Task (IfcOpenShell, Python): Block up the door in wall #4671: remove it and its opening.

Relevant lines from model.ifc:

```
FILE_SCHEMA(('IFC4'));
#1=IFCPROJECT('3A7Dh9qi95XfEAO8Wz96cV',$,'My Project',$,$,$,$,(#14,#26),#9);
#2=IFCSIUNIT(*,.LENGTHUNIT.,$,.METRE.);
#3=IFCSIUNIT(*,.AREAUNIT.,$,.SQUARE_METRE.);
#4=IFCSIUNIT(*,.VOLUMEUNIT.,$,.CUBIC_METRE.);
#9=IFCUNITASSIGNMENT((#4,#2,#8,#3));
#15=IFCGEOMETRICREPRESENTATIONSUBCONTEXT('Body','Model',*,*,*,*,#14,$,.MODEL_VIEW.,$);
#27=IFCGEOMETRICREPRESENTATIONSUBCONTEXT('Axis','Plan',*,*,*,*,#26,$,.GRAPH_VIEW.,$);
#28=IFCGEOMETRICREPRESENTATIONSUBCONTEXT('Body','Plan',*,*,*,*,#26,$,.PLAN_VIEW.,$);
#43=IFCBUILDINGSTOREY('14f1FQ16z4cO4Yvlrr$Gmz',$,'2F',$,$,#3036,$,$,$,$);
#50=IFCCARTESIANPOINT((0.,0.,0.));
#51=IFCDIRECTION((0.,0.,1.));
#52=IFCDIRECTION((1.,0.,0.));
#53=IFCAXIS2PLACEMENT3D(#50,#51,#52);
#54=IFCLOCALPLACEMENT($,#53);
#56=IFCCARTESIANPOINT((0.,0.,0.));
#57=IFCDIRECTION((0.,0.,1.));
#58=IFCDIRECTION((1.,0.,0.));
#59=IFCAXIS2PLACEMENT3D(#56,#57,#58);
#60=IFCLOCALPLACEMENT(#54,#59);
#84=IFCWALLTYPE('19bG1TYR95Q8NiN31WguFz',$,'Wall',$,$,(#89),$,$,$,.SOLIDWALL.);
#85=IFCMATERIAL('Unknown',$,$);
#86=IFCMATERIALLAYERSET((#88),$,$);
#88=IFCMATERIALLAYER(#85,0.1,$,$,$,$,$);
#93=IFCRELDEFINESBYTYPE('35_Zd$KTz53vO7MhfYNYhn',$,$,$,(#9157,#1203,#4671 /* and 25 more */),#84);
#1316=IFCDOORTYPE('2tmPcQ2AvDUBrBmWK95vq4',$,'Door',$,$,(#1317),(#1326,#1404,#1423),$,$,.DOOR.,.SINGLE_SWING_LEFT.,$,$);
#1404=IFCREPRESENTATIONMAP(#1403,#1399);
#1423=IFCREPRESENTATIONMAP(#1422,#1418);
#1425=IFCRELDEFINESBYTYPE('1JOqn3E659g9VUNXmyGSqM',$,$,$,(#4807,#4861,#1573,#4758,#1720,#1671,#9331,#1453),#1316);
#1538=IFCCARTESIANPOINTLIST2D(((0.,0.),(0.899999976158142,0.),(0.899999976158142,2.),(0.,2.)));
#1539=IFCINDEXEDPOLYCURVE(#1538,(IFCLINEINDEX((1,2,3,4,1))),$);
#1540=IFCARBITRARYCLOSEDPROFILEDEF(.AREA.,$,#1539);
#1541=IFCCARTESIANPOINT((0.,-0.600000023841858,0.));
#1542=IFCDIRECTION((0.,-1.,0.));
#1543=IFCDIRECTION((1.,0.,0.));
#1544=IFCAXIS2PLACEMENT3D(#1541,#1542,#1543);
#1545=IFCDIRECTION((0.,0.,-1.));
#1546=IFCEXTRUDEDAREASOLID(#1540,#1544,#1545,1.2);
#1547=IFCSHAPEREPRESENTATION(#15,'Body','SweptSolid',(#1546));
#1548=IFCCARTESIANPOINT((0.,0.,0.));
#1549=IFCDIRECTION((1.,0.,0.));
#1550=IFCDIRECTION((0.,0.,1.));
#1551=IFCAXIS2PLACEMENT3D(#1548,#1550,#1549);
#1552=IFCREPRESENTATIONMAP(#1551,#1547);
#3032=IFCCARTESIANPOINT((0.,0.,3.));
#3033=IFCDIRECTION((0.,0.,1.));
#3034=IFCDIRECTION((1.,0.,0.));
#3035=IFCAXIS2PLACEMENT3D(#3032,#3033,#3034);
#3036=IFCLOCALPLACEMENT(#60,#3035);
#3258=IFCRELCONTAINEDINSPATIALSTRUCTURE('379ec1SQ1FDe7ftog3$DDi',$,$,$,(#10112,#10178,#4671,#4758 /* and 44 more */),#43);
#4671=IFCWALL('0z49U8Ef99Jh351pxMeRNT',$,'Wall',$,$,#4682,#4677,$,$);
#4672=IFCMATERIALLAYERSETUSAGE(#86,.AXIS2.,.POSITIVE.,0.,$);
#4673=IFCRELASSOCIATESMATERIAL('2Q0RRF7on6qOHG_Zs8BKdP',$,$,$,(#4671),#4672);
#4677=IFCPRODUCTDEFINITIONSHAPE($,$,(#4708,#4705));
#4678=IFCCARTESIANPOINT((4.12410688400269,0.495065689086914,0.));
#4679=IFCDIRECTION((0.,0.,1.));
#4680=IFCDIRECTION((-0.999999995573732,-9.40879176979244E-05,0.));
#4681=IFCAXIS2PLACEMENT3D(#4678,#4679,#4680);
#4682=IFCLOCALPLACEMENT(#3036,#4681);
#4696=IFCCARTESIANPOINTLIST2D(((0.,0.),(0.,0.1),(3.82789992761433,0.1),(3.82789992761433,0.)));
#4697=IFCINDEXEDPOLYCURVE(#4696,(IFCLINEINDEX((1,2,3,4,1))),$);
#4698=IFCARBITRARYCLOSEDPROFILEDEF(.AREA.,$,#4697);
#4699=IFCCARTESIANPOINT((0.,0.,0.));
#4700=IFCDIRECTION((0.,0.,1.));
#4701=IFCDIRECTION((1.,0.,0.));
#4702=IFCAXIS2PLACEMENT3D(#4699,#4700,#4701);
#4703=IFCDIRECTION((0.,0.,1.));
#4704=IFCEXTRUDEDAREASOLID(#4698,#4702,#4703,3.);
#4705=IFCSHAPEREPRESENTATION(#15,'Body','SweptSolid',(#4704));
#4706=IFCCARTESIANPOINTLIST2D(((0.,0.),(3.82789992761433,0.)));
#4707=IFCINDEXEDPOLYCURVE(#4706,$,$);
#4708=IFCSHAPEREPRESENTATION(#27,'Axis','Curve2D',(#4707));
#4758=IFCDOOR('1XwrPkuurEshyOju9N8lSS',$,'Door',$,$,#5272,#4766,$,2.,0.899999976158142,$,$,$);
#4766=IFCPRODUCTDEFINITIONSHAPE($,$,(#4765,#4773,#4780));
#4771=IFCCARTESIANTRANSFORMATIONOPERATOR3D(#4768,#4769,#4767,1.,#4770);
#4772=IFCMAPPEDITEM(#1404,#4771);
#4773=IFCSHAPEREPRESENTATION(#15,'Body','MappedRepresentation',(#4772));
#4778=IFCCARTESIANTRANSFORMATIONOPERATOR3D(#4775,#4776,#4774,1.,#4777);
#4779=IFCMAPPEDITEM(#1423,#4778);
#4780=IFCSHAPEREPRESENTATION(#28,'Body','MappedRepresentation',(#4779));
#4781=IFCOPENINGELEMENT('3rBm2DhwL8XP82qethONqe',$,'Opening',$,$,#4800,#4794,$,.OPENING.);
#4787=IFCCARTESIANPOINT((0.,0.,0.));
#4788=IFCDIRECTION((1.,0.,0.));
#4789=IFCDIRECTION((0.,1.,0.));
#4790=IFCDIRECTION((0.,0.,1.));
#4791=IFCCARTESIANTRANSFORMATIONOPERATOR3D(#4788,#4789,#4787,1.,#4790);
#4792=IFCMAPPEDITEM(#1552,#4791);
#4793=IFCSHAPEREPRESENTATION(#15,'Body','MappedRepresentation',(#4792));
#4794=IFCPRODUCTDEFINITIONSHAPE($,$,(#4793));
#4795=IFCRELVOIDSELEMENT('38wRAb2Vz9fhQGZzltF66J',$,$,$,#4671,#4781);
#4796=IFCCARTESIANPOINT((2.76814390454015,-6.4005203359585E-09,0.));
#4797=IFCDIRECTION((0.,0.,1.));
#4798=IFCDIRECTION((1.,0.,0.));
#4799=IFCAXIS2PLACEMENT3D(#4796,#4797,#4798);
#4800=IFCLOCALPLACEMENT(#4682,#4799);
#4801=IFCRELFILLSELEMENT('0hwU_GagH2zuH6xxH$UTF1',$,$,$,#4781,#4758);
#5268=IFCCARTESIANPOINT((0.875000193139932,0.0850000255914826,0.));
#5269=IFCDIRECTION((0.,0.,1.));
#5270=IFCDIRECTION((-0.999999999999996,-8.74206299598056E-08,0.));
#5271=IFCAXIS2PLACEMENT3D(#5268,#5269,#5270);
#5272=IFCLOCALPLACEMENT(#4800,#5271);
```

```python
import ifcopenshell
import ifcopenshell.api.feature
import ifcopenshell.api.root
import ifcopenshell.geom
import ifcopenshell.util.shape

model = ifcopenshell.open("model.ifc")
settings = ifcopenshell.geom.settings()


def volume(element):
    """Net volume in cubic metres, openings subtracted."""
    shape = ifcopenshell.geom.create_shape(settings, element)
    return ifcopenshell.util.shape.get_volume(shape.geometry)


door = model.by_guid("1XwrPkuurEshyOju9N8lSS")
opening = door.FillsVoids[0].RelatingOpeningElement
wall = opening.VoidsElements[0].RelatingBuildingElement
before = volume(wall)

ifcopenshell.api.root.remove_product(model, product=door)
ifcopenshell.api.feature.remove_feature(model, feature=opening)

after = volume(wall)

print(f"wall volume {before:.3f} -> {after:.3f} m3")

model.write("model_edited.ifc")
```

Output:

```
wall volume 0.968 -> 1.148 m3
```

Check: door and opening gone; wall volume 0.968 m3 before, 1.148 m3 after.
